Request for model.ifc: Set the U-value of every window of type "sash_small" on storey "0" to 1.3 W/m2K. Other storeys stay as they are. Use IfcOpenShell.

First a look at what the model holds.

```python
import ifcopenshell
import ifcopenshell.util.element

model = ifcopenshell.open("model.ifc")
print(model.schema)
storey = next(s for s in model.by_type("IfcBuildingStorey") if s.Name == "0")
windows = [e for e in ifcopenshell.util.element.get_decomposition(storey) if e.is_a("IfcWindow")]
seen = {}
for e in windows:
    element_type = ifcopenshell.util.element.get_type(e)
    key = (element_type.Name if element_type != e and element_type else None, ifcopenshell.util.element.get_pset(e, "Pset_WindowCommon", "ThermalTransmittance"))
    seen[key] = seen.get(key, 0) + 1
for (name, value), count in sorted(seen.items(), key=str):
    print(count, "x", name, "|", value)
```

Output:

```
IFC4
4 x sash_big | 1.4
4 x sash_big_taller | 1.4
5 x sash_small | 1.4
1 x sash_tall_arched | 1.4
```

```python
import ifcopenshell
import ifcopenshell.api.pset
import ifcopenshell.util.element

model = ifcopenshell.open("model.ifc")

storey = next(s for s in model.by_type("IfcBuildingStorey") if s.Name == "0")
windows = [e for e in ifcopenshell.util.element.get_decomposition(storey) if e.is_a("IfcWindow")]

count = 0
for e in windows:
    element_type = ifcopenshell.util.element.get_type(e)
    if element_type in (None, e) or element_type.Name != "sash_small":
        continue
    # add_pset returns the element's existing set when there is one.
    pset = ifcopenshell.api.pset.add_pset(model, product=e, name="Pset_WindowCommon")
    ifcopenshell.api.pset.edit_pset(model, pset=pset, properties={"ThermalTransmittance": 1.3})
    count += 1

print(count, "windows updated")

model.write("model_edited.ifc")
```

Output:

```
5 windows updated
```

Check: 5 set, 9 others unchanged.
